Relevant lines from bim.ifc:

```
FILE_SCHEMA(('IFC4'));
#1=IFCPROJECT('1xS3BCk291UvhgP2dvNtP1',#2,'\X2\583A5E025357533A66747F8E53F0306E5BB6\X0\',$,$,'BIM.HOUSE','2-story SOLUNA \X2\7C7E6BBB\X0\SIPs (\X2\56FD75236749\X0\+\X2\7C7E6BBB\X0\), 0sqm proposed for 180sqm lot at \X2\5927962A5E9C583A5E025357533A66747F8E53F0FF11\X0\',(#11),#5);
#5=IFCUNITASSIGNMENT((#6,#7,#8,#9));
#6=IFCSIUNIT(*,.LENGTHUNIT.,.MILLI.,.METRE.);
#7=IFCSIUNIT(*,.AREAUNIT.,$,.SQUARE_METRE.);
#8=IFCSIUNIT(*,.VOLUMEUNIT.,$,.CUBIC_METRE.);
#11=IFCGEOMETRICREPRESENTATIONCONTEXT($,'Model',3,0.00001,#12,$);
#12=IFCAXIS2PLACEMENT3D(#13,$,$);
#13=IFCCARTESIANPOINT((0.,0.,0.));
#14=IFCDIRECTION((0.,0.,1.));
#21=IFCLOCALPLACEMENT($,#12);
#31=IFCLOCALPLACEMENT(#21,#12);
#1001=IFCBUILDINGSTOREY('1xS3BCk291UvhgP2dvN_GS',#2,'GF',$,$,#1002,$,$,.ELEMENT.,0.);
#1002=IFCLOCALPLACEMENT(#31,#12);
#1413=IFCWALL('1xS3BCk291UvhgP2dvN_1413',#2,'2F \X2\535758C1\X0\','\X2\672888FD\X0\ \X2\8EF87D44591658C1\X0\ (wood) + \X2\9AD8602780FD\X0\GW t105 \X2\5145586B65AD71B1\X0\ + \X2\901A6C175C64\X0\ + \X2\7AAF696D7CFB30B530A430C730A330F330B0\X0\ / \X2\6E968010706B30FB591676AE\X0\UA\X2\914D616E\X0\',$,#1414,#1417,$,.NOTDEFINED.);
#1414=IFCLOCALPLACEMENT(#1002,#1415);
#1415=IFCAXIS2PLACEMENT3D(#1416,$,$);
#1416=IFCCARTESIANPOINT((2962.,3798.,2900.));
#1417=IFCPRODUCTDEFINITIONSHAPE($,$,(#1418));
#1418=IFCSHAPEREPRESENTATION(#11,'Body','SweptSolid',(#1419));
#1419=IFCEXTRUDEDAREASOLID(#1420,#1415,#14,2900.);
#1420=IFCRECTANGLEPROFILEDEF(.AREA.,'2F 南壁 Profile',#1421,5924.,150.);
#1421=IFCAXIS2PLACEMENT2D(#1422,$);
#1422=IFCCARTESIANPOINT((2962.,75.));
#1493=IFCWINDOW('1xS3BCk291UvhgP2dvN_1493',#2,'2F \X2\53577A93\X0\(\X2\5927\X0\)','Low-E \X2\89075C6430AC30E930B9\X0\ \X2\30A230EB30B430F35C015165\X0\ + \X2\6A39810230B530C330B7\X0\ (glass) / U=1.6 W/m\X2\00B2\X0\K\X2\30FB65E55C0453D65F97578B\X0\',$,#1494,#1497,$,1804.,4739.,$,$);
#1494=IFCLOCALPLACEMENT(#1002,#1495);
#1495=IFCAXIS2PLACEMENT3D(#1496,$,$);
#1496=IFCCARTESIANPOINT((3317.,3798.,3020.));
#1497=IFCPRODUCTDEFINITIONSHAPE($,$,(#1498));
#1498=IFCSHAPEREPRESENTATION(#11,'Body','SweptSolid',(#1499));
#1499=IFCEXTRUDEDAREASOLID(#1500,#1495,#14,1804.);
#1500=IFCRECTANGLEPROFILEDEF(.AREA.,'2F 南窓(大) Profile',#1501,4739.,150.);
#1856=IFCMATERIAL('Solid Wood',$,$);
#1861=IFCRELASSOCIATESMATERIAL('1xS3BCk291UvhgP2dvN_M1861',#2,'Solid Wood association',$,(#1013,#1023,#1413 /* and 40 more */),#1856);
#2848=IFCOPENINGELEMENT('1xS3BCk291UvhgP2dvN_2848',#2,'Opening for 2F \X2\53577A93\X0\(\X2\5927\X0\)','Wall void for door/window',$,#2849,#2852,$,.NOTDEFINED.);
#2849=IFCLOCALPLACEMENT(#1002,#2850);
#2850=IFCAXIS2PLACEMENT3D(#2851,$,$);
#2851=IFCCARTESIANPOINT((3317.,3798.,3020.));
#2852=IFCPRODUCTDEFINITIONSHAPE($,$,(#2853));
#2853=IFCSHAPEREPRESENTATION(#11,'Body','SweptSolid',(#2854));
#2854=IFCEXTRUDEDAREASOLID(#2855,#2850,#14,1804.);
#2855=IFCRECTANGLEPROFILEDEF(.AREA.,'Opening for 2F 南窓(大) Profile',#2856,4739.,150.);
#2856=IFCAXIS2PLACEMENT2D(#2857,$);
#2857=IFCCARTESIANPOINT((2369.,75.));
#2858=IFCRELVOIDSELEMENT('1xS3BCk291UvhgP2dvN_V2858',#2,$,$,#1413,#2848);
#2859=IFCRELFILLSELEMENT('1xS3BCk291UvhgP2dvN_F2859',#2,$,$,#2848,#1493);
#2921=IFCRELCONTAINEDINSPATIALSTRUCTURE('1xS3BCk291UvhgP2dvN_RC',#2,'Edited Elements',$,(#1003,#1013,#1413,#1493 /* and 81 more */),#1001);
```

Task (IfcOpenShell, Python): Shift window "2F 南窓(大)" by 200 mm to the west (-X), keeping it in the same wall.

```python
import ifcopenshell
import ifcopenshell.api.geometry
import ifcopenshell.util.placement

model = ifcopenshell.open("bim.ifc")

window = model.by_guid("1xS3BCk291UvhgP2dvN_1493")
opening = window.FillsVoids[0].RelatingOpeningElement
wall = opening.VoidsElements[0].RelatingBuildingElement

wall_matrix = ifcopenshell.util.placement.get_local_placement(wall.ObjectPlacement)
shift = wall_matrix[:3, 0] * -200.0
before = ifcopenshell.util.placement.get_local_placement(window.ObjectPlacement)[:3, 3].copy()

# The window is not placed relative to its opening, so move both.
for product in (opening, window):
    matrix = ifcopenshell.util.placement.get_local_placement(product.ObjectPlacement)
    matrix[:3, 3] += shift
    ifcopenshell.api.geometry.edit_object_placement(model, product=product, matrix=matrix, is_si=False)

after = ifcopenshell.util.placement.get_local_placement(window.ObjectPlacement)[:3, 3]
print("window moved by", (after - before).round(3) + 0.0)

model.write("bim_rev.ifc")
```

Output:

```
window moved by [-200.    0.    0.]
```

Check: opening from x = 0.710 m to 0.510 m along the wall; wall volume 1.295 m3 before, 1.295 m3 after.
